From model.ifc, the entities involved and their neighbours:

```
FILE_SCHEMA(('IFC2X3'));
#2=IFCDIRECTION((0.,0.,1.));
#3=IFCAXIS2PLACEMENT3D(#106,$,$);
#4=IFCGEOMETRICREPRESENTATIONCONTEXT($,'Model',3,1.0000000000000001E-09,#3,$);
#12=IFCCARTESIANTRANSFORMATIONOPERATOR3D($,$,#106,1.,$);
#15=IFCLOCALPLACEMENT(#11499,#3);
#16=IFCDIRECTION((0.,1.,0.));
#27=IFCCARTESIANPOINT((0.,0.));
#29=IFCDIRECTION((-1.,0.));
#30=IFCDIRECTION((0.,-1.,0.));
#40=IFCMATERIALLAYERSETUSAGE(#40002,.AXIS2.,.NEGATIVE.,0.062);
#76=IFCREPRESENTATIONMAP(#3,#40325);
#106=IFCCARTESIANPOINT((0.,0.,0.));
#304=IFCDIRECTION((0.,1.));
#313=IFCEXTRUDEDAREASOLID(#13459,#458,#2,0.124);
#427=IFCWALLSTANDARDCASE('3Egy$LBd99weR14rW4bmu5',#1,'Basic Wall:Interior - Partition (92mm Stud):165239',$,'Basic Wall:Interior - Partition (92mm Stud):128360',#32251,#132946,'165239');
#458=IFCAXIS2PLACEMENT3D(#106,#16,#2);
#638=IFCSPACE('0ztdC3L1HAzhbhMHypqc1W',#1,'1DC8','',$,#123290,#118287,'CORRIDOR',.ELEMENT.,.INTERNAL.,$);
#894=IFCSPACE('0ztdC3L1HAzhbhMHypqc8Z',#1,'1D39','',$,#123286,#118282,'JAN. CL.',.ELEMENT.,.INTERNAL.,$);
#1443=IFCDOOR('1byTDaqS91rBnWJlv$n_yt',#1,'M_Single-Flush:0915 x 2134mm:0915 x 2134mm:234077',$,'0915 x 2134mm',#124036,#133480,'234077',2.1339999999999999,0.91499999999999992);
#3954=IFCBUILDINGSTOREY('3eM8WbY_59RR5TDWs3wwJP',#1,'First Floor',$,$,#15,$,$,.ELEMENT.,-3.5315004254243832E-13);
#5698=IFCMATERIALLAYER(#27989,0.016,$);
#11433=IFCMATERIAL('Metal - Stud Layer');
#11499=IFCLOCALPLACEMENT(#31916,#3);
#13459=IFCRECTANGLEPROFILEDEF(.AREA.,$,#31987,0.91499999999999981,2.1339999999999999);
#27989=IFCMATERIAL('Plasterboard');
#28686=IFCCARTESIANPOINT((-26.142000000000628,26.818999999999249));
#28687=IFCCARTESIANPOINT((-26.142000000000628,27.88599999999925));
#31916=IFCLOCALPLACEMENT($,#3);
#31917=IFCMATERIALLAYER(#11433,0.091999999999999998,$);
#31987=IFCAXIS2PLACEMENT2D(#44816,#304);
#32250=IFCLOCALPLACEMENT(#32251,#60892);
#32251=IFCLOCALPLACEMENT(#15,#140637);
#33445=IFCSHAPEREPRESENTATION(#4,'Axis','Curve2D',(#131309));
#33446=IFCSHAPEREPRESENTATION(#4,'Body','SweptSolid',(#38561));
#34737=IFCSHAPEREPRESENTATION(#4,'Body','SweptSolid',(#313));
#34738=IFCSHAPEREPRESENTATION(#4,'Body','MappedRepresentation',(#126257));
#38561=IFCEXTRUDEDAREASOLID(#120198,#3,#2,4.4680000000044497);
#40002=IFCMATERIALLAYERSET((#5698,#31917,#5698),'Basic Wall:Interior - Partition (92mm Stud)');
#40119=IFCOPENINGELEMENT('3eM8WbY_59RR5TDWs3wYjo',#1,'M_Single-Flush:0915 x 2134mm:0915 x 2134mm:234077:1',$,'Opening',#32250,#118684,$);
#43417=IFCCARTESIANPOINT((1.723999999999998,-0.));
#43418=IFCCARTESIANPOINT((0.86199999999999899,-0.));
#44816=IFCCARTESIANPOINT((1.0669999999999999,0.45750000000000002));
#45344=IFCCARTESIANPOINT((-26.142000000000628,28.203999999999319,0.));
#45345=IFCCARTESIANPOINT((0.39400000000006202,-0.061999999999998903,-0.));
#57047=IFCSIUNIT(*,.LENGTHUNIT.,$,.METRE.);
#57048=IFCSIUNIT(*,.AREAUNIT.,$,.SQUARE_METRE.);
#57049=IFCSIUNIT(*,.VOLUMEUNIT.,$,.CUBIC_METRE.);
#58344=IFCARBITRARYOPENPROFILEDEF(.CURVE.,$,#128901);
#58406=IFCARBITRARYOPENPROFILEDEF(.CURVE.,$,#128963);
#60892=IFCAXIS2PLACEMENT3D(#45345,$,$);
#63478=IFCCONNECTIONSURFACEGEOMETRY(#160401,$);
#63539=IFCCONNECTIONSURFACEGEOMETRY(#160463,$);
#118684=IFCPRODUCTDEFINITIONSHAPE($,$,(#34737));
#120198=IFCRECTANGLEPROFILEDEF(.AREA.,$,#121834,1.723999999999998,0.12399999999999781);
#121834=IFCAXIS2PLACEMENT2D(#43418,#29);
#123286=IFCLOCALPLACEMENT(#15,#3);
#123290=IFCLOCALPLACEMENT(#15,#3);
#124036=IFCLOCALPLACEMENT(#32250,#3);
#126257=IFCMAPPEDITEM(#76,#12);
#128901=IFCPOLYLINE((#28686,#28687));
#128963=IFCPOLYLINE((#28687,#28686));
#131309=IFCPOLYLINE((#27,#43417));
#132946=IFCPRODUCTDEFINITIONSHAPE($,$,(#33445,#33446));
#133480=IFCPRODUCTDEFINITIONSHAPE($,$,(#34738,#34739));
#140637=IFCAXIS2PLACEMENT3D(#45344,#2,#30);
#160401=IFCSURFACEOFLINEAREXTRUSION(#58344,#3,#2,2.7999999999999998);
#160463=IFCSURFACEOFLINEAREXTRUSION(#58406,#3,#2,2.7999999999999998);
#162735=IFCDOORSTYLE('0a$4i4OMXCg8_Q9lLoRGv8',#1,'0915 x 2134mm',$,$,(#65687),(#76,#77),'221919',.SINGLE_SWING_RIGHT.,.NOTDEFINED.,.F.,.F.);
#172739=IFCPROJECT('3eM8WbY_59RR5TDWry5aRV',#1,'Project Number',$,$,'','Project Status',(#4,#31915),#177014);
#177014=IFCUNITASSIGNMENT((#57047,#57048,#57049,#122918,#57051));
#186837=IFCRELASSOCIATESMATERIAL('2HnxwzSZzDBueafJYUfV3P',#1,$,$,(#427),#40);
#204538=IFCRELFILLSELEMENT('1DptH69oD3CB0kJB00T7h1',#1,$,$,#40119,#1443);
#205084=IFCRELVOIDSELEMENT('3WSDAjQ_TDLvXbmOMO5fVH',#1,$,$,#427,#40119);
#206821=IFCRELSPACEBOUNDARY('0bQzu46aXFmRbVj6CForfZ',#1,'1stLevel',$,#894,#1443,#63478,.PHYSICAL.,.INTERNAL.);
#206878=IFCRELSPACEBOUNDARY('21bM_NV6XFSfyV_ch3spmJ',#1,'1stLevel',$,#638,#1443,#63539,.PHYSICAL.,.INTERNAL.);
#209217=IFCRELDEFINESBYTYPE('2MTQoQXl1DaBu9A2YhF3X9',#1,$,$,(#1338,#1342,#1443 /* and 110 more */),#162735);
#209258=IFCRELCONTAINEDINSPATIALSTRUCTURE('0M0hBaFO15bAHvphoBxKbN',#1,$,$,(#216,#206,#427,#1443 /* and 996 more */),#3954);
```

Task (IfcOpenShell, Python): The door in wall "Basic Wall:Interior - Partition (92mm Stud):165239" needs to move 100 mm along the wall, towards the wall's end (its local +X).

```python
import numpy as np
import ifcopenshell
import ifcopenshell.api.geometry
import ifcopenshell.util.placement
import ifcopenshell.util.unit

model = ifcopenshell.open("model.ifc")
unit_scale = ifcopenshell.util.unit.calculate_unit_scale(model)

door = model.by_guid("1byTDaqS91rBnWJlv$n_yt")
opening = door.FillsVoids[0].RelatingOpeningElement
wall = opening.VoidsElements[0].RelatingBuildingElement

wall_matrix = ifcopenshell.util.placement.get_local_placement(wall.ObjectPlacement)
shift = wall_matrix[:3, 0] * 0.1 / unit_scale
before = ifcopenshell.util.placement.get_local_placement(door.ObjectPlacement)[:3, 3].copy()

# The door is placed relative to its opening, so it follows when the opening moves.
matrix = ifcopenshell.util.placement.get_local_placement(opening.ObjectPlacement)
matrix[:3, 3] += shift
ifcopenshell.api.geometry.edit_object_placement(
    model, product=opening, matrix=matrix, is_si=False, should_transform_children=True
)

# Space boundary surfaces are stored in each space's coordinates; move them too.
for rel in door.ProvidesBoundaries:
    if not rel.ConnectionGeometry:
        continue
    surface = rel.ConnectionGeometry.SurfaceOnRelatingElement
    space_matrix = ifcopenshell.util.placement.get_local_placement(rel.RelatingSpace.ObjectPlacement)
    point = np.array(surface.Position.Location.Coordinates) + space_matrix[:3, :3].T @ shift
    surface.Position = model.createIfcAxis2Placement3D(
        model.createIfcCartesianPoint(point.tolist()), surface.Position.Axis, surface.Position.RefDirection
    )

after = ifcopenshell.util.placement.get_local_placement(door.ObjectPlacement)[:3, 3]
print("door moved by", (after - before).round(3) + 0.0)

model.write("model_edited.ifc")
```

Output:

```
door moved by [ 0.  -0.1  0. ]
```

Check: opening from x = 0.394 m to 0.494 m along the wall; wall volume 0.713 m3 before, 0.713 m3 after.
